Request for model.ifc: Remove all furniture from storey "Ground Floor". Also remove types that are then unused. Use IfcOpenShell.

First a look at what the model holds.

```python
import ifcopenshell
import ifcopenshell.util.element

model = ifcopenshell.open("model.ifc")
print(model.schema)
storey = next(s for s in model.by_type("IfcBuildingStorey") if s.Name == "Ground Floor")
furniture = [e for e in ifcopenshell.util.element.get_decomposition(storey) if e.is_a("IfcFurnishingElement")]
seen = {}
for e in furniture:
    element_type = ifcopenshell.util.element.get_type(e)
    name = element_type.Name if element_type not in (None, e) else None
    seen[name] = seen.get(name, 0) + 1
for name, count in sorted(seen.items(), key=str):
    print(count, "x", name)
```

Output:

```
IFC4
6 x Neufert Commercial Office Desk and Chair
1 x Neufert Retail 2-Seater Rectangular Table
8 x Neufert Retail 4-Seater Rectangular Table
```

```python
import ifcopenshell
import ifcopenshell.api.root
import ifcopenshell.util.element

model = ifcopenshell.open("model.ifc")

storey = next(s for s in model.by_type("IfcBuildingStorey") if s.Name == "Ground Floor")
furniture = [e for e in ifcopenshell.util.element.get_decomposition(storey) if e.is_a("IfcFurnishingElement")]
types = {ifcopenshell.util.element.get_type(e) for e in furniture} - {None, *furniture}

for e in furniture:
    ifcopenshell.api.root.remove_product(model, product=e)
print(len(furniture), "removed")

unused = [t for t in types if not ifcopenshell.util.element.get_types(t)]
for t in unused:
    ifcopenshell.api.root.remove_product(model, product=t)
print(len(unused), "unused types removed")

model.write("model_updated.ifc")
```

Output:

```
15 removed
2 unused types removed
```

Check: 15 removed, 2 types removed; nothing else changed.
